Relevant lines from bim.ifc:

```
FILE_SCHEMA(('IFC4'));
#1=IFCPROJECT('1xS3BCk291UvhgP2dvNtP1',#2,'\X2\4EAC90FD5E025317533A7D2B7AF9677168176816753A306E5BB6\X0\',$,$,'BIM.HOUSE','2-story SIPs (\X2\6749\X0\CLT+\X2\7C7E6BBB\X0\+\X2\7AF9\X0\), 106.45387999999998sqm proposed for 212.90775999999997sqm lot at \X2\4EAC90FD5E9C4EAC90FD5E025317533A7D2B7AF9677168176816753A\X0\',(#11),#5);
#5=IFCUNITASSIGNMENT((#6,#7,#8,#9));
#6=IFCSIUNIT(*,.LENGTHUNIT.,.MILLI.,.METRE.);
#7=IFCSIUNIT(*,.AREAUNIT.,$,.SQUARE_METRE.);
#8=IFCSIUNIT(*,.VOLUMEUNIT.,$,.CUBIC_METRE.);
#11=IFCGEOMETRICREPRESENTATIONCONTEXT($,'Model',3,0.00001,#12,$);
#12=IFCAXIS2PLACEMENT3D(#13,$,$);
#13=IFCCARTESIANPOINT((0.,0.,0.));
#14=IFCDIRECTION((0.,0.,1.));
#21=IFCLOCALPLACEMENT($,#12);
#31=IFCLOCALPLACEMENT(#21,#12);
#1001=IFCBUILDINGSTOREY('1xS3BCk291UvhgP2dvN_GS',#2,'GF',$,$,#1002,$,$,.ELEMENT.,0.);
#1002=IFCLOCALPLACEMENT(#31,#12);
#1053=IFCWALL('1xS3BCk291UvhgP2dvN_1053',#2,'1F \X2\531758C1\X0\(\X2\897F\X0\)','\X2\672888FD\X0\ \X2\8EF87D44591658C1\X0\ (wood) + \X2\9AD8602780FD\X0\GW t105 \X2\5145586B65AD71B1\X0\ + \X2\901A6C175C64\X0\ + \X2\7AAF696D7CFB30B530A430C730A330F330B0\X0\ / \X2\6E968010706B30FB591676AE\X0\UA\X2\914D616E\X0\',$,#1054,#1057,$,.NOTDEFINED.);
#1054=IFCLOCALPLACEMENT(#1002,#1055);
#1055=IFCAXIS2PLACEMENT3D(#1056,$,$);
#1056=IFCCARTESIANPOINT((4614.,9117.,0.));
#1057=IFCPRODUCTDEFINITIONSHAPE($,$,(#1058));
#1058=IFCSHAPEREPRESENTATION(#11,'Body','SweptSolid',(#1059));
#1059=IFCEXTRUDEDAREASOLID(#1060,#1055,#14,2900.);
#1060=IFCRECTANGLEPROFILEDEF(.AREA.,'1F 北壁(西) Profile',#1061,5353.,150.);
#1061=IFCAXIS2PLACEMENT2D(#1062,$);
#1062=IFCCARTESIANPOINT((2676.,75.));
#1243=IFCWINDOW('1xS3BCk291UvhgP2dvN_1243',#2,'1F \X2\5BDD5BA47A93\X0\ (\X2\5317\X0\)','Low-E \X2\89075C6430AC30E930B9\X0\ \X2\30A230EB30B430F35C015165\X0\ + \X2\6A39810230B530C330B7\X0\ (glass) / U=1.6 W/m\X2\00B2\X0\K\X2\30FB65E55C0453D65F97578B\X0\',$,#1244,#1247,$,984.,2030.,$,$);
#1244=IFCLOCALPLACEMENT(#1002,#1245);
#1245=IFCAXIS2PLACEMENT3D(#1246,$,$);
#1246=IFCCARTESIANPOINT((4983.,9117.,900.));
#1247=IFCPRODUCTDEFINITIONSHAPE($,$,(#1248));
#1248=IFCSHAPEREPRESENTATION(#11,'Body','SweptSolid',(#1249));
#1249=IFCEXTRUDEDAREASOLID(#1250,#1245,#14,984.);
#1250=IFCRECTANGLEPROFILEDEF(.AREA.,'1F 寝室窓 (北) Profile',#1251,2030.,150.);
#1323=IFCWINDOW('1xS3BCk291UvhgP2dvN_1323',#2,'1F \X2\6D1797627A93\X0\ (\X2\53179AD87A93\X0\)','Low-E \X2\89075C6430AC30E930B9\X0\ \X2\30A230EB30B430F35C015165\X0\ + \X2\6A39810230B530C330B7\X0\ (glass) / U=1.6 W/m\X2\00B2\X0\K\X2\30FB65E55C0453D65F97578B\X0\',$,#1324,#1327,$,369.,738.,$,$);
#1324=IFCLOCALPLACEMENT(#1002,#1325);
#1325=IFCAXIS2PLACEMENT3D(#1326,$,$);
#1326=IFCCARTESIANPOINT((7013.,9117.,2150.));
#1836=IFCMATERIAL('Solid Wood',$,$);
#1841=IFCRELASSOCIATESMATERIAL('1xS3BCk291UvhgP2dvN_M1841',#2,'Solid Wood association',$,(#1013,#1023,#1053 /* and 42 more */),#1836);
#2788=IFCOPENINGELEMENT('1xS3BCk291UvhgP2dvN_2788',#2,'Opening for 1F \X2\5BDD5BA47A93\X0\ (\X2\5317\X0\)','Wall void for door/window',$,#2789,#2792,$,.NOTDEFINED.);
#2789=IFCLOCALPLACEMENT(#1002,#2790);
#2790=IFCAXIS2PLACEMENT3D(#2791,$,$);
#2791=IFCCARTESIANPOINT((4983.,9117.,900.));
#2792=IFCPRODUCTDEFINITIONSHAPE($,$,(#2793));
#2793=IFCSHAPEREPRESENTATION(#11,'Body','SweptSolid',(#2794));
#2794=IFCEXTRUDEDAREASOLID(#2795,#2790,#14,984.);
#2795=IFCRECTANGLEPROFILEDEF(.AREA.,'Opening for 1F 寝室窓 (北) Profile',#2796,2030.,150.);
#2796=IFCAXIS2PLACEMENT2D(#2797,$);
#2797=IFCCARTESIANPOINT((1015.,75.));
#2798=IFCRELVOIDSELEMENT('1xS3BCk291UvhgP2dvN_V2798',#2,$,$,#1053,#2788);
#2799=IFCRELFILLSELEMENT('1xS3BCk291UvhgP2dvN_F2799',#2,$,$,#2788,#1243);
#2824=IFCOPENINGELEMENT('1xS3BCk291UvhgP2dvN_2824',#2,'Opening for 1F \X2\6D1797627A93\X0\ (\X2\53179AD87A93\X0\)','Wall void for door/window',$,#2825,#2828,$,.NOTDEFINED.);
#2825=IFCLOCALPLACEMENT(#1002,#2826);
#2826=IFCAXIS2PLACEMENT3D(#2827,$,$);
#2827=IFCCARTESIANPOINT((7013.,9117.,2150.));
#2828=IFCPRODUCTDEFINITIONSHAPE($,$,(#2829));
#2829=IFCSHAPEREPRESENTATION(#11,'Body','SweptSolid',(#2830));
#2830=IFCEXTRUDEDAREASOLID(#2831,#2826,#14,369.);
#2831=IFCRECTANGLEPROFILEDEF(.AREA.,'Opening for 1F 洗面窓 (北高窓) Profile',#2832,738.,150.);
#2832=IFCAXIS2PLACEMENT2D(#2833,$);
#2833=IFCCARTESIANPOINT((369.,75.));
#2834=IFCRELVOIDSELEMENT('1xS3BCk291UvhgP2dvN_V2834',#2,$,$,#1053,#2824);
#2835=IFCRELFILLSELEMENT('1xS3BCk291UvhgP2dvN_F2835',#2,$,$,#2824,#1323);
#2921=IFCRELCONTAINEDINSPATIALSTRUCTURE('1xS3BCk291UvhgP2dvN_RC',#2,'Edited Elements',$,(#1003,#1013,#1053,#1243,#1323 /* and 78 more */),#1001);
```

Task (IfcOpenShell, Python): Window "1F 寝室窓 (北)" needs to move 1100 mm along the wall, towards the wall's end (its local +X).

```python
import ifcopenshell
import ifcopenshell.api.geometry
import ifcopenshell.util.placement
import ifcopenshell.util.unit

model = ifcopenshell.open("bim.ifc")
unit_scale = ifcopenshell.util.unit.calculate_unit_scale(model)

window = model.by_id(1243)
opening = window.FillsVoids[0].RelatingOpeningElement
wall = opening.VoidsElements[0].RelatingBuildingElement

wall_matrix = ifcopenshell.util.placement.get_local_placement(wall.ObjectPlacement)
shift = wall_matrix[:3, 0] * 1.1 / unit_scale
before = ifcopenshell.util.placement.get_local_placement(window.ObjectPlacement)[:3, 3].copy()

# The window is not placed relative to its opening, so move both.
for product in (opening, window):
    matrix = ifcopenshell.util.placement.get_local_placement(product.ObjectPlacement)
    matrix[:3, 3] += shift
    ifcopenshell.api.geometry.edit_object_placement(model, product=product, matrix=matrix, is_si=False)

after = ifcopenshell.util.placement.get_local_placement(window.ObjectPlacement)[:3, 3]
print("window moved by", (after - before).round(3) + 0.0)

model.write("bim_v2.ifc")
```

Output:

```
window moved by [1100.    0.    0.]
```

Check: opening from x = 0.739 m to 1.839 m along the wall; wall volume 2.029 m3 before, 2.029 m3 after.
